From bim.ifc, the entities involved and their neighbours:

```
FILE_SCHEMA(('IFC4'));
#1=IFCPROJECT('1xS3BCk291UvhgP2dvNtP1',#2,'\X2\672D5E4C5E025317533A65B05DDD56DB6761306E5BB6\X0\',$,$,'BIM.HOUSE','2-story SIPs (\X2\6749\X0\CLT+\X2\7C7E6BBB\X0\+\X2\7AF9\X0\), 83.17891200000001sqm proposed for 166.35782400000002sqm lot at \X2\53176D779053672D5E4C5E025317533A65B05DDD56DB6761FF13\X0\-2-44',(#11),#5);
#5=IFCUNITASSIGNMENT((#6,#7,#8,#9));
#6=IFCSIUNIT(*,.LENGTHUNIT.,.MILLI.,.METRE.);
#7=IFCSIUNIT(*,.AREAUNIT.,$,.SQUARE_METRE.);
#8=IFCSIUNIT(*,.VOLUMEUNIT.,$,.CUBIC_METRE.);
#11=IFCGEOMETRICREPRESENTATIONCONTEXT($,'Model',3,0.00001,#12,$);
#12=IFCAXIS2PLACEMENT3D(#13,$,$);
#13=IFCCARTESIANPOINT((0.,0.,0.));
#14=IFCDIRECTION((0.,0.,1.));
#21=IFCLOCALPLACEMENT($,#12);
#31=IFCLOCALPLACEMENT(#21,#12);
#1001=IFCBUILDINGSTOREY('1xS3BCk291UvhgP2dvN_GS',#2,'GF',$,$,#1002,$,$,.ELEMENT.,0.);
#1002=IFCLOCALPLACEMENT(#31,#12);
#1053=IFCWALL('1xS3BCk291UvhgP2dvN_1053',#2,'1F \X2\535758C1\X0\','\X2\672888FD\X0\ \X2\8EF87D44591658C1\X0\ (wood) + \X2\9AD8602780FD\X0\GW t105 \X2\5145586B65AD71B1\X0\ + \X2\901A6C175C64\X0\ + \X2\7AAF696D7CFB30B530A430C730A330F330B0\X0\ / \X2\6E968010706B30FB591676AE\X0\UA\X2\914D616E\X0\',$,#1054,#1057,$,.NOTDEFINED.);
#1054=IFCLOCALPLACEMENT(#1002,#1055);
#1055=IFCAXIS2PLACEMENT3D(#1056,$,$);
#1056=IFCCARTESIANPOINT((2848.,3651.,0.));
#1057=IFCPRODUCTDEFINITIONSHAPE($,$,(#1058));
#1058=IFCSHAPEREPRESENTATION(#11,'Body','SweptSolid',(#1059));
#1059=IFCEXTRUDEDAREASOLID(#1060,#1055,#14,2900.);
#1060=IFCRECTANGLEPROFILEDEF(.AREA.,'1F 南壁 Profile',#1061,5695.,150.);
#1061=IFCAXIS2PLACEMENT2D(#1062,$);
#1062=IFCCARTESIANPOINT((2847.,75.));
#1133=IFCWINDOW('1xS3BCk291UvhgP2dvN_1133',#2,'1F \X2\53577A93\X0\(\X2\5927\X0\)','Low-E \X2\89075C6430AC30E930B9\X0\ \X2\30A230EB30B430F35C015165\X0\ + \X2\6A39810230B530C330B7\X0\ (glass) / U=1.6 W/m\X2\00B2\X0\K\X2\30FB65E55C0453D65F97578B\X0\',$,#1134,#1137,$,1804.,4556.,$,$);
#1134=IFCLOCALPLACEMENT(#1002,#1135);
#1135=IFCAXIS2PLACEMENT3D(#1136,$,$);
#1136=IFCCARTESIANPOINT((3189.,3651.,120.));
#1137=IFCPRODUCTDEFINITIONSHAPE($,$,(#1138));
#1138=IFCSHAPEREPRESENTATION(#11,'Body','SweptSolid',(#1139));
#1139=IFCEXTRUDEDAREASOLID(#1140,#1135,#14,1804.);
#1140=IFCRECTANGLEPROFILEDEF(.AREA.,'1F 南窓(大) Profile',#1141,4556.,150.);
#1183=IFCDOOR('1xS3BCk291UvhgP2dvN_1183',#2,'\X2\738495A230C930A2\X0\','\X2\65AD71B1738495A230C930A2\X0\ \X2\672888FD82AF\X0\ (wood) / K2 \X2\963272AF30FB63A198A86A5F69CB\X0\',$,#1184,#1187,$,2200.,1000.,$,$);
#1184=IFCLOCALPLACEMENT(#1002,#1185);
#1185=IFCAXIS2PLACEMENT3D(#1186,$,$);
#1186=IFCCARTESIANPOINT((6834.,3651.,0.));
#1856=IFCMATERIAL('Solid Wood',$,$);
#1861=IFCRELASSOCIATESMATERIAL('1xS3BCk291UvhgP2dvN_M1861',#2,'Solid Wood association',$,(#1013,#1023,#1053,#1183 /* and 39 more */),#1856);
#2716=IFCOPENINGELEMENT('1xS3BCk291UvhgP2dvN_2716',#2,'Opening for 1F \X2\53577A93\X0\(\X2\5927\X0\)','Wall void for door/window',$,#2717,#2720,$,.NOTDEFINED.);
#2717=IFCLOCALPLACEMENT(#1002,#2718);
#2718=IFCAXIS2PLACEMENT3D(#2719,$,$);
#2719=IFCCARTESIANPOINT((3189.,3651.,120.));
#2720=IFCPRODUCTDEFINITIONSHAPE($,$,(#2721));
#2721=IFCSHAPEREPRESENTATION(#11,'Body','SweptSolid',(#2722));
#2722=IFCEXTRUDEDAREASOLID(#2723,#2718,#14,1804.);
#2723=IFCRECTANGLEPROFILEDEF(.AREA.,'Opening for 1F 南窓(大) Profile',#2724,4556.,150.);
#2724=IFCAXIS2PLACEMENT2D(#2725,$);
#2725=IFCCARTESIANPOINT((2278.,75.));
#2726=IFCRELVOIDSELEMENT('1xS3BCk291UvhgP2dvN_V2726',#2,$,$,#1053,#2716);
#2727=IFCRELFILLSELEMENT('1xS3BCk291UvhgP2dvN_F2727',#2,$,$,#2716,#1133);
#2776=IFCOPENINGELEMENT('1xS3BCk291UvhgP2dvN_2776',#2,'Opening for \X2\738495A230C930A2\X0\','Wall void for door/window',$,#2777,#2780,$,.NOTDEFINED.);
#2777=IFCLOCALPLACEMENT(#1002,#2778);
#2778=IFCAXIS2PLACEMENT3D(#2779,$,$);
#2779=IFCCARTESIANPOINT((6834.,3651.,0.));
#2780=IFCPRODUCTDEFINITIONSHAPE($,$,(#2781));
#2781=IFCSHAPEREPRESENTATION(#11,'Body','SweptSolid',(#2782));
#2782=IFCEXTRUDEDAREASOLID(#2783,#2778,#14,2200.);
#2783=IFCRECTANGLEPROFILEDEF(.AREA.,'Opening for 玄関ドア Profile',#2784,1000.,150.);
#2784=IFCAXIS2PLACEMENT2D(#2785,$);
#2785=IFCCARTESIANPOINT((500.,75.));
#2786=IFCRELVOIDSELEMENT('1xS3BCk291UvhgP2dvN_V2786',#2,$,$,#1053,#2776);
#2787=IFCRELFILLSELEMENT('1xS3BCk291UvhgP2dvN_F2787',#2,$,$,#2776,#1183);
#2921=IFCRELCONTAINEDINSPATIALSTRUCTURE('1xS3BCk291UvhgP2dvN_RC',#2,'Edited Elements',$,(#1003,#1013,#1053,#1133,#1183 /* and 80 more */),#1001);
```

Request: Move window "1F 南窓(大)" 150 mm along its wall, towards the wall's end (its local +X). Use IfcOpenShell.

```python
import ifcopenshell
import ifcopenshell.api.geometry
import ifcopenshell.util.placement
import ifcopenshell.util.unit

model = ifcopenshell.open("bim.ifc")
unit_scale = ifcopenshell.util.unit.calculate_unit_scale(model)

window = model.by_guid("1xS3BCk291UvhgP2dvN_1133")
opening = window.FillsVoids[0].RelatingOpeningElement
wall = opening.VoidsElements[0].RelatingBuildingElement

wall_matrix = ifcopenshell.util.placement.get_local_placement(wall.ObjectPlacement)
shift = wall_matrix[:3, 0] * 0.15 / unit_scale
before = ifcopenshell.util.placement.get_local_placement(window.ObjectPlacement)[:3, 3].copy()

# The window is not placed relative to its opening, so move both.
for product in (opening, window):
    matrix = ifcopenshell.util.placement.get_local_placement(product.ObjectPlacement)
    matrix[:3, 3] += shift
    ifcopenshell.api.geometry.edit_object_placement(model, product=product, matrix=matrix, is_si=False)

after = ifcopenshell.util.placement.get_local_placement(window.ObjectPlacement)[:3, 3]
print("window moved by", (after - before).round(3) + 0.0)

model.write("bim-out.ifc")
```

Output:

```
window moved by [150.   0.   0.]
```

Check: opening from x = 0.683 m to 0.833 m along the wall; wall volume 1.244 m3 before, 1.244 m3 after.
